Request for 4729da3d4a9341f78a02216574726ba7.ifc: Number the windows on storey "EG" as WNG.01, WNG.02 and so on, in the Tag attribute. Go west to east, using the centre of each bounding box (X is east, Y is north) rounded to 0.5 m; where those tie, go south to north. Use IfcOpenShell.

First a look at what the model holds.

```python
import ifcopenshell
import ifcopenshell.util.element
import ifcopenshell.util.placement

model = ifcopenshell.open("4729da3d4a9341f78a02216574726ba7.ifc")
print(model.schema)
storey = next(s for s in model.by_type("IfcBuildingStorey") if s.Name == "EG")
windows = [e for e in ifcopenshell.util.element.get_decomposition(storey) if e.is_a("IfcWindow")]
for e in sorted(windows, key=lambda e: e.id()):
    origin = ifcopenshell.util.placement.get_local_placement(e.ObjectPlacement)[:3, 3]
    print(e.id(), e.Tag, e.Name, origin.round(2) + 0.0, sep=" | ")
```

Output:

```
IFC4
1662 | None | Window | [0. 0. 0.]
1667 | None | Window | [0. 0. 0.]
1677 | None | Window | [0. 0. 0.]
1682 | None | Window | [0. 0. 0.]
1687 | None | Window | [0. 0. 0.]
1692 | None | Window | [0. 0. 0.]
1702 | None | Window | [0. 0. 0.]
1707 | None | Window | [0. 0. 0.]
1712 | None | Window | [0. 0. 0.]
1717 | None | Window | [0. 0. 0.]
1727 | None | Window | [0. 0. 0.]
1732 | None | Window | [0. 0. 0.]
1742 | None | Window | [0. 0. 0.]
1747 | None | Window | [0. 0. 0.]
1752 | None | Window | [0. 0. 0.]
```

```python
import ifcopenshell
import ifcopenshell.geom
import ifcopenshell.util.element
import ifcopenshell.util.shape

model = ifcopenshell.open("4729da3d4a9341f78a02216574726ba7.ifc")
settings = ifcopenshell.geom.settings()
settings.set("use-world-coords", True)


def centre(element):
    shape = ifcopenshell.geom.create_shape(settings, element)
    return ifcopenshell.util.shape.get_bbox_centroid(shape.geometry)


storey = next(s for s in model.by_type("IfcBuildingStorey") if s.Name == "EG")
windows = [e for e in ifcopenshell.util.element.get_decomposition(storey) if e.is_a("IfcWindow")]

# Insertion points can sit at a corner or the storey origin, so sort by the geometry (in metres).
centres = {e: centre(e) for e in windows}
windows.sort(key=lambda e: (round(centres[e][0] / 0.5), centres[e][1]))

for i, e in enumerate(windows, start=1):
    number = f"WNG.{i:02d}"
    e.Tag = number
    print(e.id(), number)

model.write("4729da3d4a9341f78a02216574726ba7_updated.ifc")
```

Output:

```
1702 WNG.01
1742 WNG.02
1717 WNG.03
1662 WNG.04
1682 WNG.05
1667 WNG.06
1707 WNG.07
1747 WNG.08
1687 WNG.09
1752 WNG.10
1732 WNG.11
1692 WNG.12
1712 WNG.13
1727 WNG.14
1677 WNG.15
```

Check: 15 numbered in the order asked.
